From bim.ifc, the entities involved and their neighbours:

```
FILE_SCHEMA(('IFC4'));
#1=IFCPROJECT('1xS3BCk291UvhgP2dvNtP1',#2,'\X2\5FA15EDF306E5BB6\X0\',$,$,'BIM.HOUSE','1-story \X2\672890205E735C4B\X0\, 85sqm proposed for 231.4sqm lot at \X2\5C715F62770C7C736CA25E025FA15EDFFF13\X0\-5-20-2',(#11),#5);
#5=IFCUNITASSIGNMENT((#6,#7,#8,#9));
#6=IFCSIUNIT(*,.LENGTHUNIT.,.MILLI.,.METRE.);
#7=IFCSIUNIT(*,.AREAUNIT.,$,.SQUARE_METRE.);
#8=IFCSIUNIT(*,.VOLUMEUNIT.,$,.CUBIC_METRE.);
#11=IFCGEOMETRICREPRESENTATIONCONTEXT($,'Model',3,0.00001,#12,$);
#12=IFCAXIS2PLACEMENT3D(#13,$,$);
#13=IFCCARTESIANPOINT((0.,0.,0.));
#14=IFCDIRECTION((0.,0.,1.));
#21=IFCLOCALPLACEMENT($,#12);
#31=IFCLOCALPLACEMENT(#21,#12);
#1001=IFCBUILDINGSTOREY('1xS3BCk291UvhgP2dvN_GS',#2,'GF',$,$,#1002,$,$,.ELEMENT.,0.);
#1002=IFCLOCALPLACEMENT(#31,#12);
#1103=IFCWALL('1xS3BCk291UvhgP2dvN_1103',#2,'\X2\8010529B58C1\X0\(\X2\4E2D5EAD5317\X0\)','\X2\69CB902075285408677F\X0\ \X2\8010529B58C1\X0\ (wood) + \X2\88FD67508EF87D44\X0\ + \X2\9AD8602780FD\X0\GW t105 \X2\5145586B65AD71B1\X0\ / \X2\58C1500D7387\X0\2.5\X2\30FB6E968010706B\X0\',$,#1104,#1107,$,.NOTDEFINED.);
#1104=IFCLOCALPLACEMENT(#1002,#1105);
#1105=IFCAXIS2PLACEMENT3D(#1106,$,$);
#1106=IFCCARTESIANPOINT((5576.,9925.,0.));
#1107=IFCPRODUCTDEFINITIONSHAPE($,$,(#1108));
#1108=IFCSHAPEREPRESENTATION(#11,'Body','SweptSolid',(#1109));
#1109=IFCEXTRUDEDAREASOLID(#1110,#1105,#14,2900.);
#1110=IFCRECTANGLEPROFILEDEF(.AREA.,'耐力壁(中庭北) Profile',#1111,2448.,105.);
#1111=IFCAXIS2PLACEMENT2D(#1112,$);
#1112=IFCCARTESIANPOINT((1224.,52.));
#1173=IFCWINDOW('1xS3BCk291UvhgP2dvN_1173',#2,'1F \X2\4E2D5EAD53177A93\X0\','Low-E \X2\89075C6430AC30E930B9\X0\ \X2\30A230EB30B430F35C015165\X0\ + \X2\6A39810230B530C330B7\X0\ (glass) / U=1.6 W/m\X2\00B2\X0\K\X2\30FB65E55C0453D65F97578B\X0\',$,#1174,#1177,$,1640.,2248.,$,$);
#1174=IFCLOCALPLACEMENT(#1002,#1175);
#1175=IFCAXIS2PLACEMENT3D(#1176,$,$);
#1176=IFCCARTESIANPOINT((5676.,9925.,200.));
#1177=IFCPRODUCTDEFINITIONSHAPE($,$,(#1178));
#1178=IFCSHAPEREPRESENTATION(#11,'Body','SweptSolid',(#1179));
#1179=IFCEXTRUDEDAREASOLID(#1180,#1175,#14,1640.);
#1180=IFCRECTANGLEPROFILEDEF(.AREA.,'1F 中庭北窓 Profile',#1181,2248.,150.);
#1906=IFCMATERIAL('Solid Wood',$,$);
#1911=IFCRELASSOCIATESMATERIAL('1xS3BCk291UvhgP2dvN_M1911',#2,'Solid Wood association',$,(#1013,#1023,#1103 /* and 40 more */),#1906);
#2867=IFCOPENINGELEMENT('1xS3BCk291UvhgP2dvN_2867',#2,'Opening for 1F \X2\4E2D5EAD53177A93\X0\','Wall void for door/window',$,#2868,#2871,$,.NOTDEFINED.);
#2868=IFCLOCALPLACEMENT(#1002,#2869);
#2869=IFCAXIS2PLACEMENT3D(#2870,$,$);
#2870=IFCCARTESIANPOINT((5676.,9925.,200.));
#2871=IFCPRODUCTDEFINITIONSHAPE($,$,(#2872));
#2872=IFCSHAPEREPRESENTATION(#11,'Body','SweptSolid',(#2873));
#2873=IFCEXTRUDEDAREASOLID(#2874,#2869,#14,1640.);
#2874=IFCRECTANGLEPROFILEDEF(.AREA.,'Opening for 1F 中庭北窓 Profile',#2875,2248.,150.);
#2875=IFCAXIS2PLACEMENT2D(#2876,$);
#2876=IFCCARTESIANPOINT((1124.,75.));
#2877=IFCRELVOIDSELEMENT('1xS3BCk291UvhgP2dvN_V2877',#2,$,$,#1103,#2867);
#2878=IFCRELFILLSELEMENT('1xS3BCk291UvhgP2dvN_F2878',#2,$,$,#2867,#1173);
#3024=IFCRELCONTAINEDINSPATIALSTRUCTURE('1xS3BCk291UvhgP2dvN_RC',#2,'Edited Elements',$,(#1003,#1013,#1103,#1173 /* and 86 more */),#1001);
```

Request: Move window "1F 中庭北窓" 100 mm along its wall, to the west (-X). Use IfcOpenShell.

```python
import ifcopenshell
import ifcopenshell.api.geometry
import ifcopenshell.util.placement
import ifcopenshell.util.unit

model = ifcopenshell.open("bim.ifc")
unit_scale = ifcopenshell.util.unit.calculate_unit_scale(model)

window = model.by_guid("1xS3BCk291UvhgP2dvN_1173")
opening = window.FillsVoids[0].RelatingOpeningElement
wall = opening.VoidsElements[0].RelatingBuildingElement

wall_matrix = ifcopenshell.util.placement.get_local_placement(wall.ObjectPlacement)
shift = wall_matrix[:3, 0] * -0.1 / unit_scale
before = ifcopenshell.util.placement.get_local_placement(window.ObjectPlacement)[:3, 3].copy()

# The window is not placed relative to its opening, so move both.
for product in (opening, window):
    matrix = ifcopenshell.util.placement.get_local_placement(product.ObjectPlacement)
    matrix[:3, 3] += shift
    ifcopenshell.api.geometry.edit_object_placement(model, product=product, matrix=matrix, is_si=False)

after = ifcopenshell.util.placement.get_local_placement(window.ObjectPlacement)[:3, 3]
print("window moved by", (after - before).round(3) + 0.0)

model.write("bim_rev.ifc")
```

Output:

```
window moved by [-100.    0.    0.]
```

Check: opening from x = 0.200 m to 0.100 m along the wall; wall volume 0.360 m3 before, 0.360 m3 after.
